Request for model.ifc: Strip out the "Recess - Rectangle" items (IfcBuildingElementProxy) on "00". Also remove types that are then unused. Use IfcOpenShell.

First a look at what the model holds.

```python
import ifcopenshell
import ifcopenshell.util.element

model = ifcopenshell.open("model.ifc")
print(model.schema)
storey = next(s for s in model.by_type("IfcBuildingStorey") if s.Name == "00")
proxies = [e for e in ifcopenshell.util.element.get_decomposition(storey) if e.is_a("IfcBuildingElementProxy")]
seen = {}
for e in proxies:
    element_type = ifcopenshell.util.element.get_type(e)
    name = element_type.Name if element_type not in (None, e) else None
    seen[name] = seen.get(name, 0) + 1
for name, count in sorted(seen.items(), key=str):
    print(count, "x", name)
```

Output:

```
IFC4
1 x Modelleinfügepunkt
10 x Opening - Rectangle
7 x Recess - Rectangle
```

```python
import ifcopenshell
import ifcopenshell.api.root
import ifcopenshell.util.element

model = ifcopenshell.open("model.ifc")

storey = next(s for s in model.by_type("IfcBuildingStorey") if s.Name == "00")
proxies = [e for e in ifcopenshell.util.element.get_decomposition(storey) if e.is_a("IfcBuildingElementProxy")]
targets = [e for e in proxies if (t := ifcopenshell.util.element.get_type(e)) not in (None, e) and t.Name == "Recess - Rectangle"]
types = {ifcopenshell.util.element.get_type(e) for e in targets} - {None, *targets}

for e in targets:
    ifcopenshell.api.root.remove_product(model, product=e)
print(len(targets), "removed")

unused = [t for t in types if not ifcopenshell.util.element.get_types(t)]
for t in unused:
    ifcopenshell.api.root.remove_product(model, product=t)
print(len(unused), "unused types removed")

model.write("model-out.ifc")
```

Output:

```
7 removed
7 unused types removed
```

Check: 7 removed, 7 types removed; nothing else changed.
